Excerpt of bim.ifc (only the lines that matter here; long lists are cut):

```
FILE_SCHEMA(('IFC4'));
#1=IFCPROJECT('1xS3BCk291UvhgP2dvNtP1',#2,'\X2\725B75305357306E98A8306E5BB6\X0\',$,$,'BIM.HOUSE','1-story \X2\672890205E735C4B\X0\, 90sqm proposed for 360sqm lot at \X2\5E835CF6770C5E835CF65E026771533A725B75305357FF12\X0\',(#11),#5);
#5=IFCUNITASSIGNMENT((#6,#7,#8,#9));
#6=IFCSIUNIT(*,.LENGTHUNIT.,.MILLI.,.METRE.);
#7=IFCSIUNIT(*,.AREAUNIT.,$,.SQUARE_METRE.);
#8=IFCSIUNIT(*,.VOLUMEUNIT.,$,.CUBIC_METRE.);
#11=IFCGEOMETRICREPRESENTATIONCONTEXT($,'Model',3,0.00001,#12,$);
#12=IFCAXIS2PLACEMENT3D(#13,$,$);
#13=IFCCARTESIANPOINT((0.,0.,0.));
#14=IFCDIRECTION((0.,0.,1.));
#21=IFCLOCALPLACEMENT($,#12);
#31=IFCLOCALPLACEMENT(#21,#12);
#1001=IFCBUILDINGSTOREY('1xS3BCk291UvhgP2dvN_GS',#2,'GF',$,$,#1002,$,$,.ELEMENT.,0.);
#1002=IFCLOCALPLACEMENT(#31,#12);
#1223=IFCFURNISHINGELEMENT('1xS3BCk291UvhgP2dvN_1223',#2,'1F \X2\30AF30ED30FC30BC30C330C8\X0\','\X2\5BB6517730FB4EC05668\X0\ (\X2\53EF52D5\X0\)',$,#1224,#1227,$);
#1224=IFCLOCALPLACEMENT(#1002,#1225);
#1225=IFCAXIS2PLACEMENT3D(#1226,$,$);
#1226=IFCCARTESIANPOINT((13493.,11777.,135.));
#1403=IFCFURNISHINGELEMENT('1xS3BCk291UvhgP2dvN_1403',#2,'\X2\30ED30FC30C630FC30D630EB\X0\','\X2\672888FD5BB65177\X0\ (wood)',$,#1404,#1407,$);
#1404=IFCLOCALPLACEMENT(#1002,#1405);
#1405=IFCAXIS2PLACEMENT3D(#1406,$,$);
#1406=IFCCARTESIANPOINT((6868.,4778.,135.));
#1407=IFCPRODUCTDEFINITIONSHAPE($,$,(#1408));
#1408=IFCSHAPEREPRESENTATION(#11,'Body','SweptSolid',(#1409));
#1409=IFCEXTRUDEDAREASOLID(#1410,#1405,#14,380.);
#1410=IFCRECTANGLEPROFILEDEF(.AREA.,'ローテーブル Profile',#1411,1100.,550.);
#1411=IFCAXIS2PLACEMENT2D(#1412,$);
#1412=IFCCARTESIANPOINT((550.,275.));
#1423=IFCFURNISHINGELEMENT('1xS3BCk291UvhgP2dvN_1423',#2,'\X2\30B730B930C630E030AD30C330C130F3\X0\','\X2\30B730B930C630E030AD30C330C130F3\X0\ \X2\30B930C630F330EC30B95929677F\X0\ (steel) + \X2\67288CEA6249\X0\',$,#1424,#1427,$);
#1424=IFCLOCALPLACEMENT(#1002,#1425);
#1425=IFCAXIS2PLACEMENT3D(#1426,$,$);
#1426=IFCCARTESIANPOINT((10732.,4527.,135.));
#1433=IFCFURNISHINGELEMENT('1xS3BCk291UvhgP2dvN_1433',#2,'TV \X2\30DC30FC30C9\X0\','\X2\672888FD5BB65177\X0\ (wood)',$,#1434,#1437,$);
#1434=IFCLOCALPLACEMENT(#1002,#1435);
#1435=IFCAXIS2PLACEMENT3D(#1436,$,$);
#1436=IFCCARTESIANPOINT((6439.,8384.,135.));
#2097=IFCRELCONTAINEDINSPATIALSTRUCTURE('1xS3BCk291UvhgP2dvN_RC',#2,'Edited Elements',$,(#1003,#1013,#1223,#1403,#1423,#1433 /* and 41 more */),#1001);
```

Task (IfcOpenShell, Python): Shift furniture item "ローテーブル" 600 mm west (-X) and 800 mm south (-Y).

```python
import ifcopenshell
import ifcopenshell.api.geometry
import ifcopenshell.util.placement
import ifcopenshell.util.unit

model = ifcopenshell.open("bim.ifc")
unit_scale = ifcopenshell.util.unit.calculate_unit_scale(model)

item = model.by_guid("1xS3BCk291UvhgP2dvN_1403")
matrix = ifcopenshell.util.placement.get_local_placement(item.ObjectPlacement)
matrix[0, 3] -= 0.6 / unit_scale
matrix[1, 3] -= 0.8 / unit_scale
ifcopenshell.api.geometry.edit_object_placement(model, product=item, matrix=matrix, is_si=False)

print(ifcopenshell.util.placement.get_local_placement(item.ObjectPlacement).round(3) + 0.0)

model.write("bim_rev.ifc")
```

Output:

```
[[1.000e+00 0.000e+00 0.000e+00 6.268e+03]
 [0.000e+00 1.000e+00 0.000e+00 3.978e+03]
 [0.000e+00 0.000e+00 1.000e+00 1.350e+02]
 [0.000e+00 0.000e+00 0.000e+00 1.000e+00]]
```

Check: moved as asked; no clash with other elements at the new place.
